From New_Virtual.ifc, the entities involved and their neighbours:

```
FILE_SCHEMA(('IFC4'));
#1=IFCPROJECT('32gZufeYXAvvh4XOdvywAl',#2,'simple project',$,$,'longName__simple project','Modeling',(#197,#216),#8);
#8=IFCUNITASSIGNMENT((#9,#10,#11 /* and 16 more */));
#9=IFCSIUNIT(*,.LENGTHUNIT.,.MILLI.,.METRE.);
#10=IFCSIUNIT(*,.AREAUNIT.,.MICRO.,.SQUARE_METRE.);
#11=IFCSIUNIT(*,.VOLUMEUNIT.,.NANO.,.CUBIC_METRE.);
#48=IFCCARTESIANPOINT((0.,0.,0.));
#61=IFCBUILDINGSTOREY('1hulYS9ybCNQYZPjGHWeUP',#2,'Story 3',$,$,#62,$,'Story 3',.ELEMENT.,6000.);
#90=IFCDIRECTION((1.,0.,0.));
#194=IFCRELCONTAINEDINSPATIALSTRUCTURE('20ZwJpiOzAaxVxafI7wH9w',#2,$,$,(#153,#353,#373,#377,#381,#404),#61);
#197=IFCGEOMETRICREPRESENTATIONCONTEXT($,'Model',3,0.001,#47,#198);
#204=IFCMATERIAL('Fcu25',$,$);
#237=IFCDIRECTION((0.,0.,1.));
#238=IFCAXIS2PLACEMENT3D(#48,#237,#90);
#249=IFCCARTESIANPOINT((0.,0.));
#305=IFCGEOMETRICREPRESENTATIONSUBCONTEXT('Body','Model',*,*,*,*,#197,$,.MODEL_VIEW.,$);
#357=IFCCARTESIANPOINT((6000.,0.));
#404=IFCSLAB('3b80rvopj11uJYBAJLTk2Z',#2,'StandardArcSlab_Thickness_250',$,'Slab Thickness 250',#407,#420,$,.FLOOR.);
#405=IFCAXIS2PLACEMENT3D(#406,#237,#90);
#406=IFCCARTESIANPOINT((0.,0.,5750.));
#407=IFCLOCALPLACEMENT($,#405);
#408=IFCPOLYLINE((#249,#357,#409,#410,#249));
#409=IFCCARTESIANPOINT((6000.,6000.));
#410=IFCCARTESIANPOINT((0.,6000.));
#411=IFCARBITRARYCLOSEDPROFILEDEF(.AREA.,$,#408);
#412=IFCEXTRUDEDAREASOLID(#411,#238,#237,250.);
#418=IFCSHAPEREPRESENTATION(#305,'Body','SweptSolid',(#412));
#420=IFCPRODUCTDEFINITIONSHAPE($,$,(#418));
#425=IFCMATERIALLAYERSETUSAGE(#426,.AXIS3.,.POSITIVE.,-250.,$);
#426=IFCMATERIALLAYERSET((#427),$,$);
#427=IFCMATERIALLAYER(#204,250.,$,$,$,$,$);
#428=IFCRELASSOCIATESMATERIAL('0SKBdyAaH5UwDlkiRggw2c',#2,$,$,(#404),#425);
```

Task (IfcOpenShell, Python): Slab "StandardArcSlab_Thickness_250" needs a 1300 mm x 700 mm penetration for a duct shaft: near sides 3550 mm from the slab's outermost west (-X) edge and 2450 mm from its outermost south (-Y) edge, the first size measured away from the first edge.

```python
import numpy as np
import ifcopenshell
import ifcopenshell.api.feature
import ifcopenshell.api.geometry
import ifcopenshell.api.root
import ifcopenshell.geom
import ifcopenshell.util.placement
import ifcopenshell.util.representation
import ifcopenshell.util.shape
import ifcopenshell.util.unit

model = ifcopenshell.open("New_Virtual.ifc")
unit_scale = ifcopenshell.util.unit.calculate_unit_scale(model)
settings = ifcopenshell.geom.settings()


def volume(element):
    """Net volume in cubic metres, openings subtracted."""
    shape = ifcopenshell.geom.create_shape(settings, element)
    return ifcopenshell.util.shape.get_volume(shape.geometry)


slab = model.by_guid("3b80rvopj11uJYBAJLTk2Z")
before = volume(slab)

# Extent in the slab's own axes, in metres. The edges named are its -X and -Y sides.
slab_shape = ifcopenshell.geom.create_shape(settings, slab)
vertices = ifcopenshell.util.shape.get_vertices(slab_shape.geometry)
x_min, y_min, bottom = vertices.min(axis=0)
top = vertices[:, 2].max()

opening = ifcopenshell.api.root.create_entity(model, ifc_class="IfcOpeningElement", name="Duct shaft opening", predefined_type="OPENING")
context = ifcopenshell.util.representation.get_context(model, "Model", "Body", "MODEL_VIEW")
width, depth = 1.3, 0.7
outline = [(0.0, 0.0), (width, 0.0), (width, depth), (0.0, depth), (0.0, 0.0)]
# Overshoot both faces by 50 mm so the cut is clean.
shape = ifcopenshell.api.geometry.add_slab_representation(
    model, context=context, depth=top - bottom + 0.1, polyline=outline
)
ifcopenshell.api.geometry.assign_representation(model, product=opening, representation=shape)

matrix = ifcopenshell.util.placement.get_local_placement(slab.ObjectPlacement)
matrix[:, 3] = matrix @ np.append(np.array([x_min + 3.55, y_min + 2.45, bottom - 0.05]) / unit_scale, 1.0)
ifcopenshell.api.geometry.edit_object_placement(model, product=opening, matrix=matrix, is_si=False)
ifcopenshell.api.feature.add_feature(model, feature=opening, element=slab)

after = volume(slab)

print(f"slab volume {before:.3f} -> {after:.3f} m3")

model.write("New_Virtual_v2.ifc")
```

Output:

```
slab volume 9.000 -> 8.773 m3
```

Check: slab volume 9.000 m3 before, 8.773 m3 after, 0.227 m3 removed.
